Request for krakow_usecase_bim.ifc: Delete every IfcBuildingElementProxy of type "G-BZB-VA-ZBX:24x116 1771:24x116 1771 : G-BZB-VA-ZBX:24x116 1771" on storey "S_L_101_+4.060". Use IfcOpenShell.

First a look at what the model holds.

```python
import ifcopenshell
import ifcopenshell.util.element

model = ifcopenshell.open("krakow_usecase_bim.ifc")
print(model.schema)
storey = next(s for s in model.by_type("IfcBuildingStorey") if s.Name == "S_L_101_+4.060")
proxies = [e for e in ifcopenshell.util.element.get_decomposition(storey) if e.is_a("IfcBuildingElementProxy")]
seen = {}
for e in proxies:
    element_type = ifcopenshell.util.element.get_type(e)
    name = element_type.Name if element_type not in (None, e) else None
    seen[name] = seen.get(name, 0) + 1
for name, count in sorted(seen.items(), key=str):
    print(count, "x", name)
```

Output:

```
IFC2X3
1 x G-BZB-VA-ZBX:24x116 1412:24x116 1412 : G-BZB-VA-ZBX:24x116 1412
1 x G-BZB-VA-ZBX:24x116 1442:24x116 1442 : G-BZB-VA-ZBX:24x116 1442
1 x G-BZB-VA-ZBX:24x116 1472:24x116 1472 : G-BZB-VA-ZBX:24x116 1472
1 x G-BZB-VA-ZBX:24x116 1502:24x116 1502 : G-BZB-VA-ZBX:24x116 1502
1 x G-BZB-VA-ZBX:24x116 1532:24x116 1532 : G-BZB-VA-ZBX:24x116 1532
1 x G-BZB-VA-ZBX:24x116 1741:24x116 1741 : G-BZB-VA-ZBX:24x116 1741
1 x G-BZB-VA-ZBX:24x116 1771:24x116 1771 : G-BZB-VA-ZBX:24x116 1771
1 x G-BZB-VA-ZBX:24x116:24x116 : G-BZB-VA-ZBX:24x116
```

```python
import ifcopenshell
import ifcopenshell.api.root
import ifcopenshell.util.element

model = ifcopenshell.open("krakow_usecase_bim.ifc")

storey = next(s for s in model.by_type("IfcBuildingStorey") if s.Name == "S_L_101_+4.060")
proxies = [e for e in ifcopenshell.util.element.get_decomposition(storey) if e.is_a("IfcBuildingElementProxy")]
targets = [e for e in proxies if (t := ifcopenshell.util.element.get_type(e)) not in (None, e) and t.Name == "G-BZB-VA-ZBX:24x116 1771:24x116 1771 : G-BZB-VA-ZBX:24x116 1771"]

for e in targets:
    ifcopenshell.api.root.remove_product(model, product=e)
print(len(targets), "removed")

model.write("krakow_usecase_bim_rev.ifc")
```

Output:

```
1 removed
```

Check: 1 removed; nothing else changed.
